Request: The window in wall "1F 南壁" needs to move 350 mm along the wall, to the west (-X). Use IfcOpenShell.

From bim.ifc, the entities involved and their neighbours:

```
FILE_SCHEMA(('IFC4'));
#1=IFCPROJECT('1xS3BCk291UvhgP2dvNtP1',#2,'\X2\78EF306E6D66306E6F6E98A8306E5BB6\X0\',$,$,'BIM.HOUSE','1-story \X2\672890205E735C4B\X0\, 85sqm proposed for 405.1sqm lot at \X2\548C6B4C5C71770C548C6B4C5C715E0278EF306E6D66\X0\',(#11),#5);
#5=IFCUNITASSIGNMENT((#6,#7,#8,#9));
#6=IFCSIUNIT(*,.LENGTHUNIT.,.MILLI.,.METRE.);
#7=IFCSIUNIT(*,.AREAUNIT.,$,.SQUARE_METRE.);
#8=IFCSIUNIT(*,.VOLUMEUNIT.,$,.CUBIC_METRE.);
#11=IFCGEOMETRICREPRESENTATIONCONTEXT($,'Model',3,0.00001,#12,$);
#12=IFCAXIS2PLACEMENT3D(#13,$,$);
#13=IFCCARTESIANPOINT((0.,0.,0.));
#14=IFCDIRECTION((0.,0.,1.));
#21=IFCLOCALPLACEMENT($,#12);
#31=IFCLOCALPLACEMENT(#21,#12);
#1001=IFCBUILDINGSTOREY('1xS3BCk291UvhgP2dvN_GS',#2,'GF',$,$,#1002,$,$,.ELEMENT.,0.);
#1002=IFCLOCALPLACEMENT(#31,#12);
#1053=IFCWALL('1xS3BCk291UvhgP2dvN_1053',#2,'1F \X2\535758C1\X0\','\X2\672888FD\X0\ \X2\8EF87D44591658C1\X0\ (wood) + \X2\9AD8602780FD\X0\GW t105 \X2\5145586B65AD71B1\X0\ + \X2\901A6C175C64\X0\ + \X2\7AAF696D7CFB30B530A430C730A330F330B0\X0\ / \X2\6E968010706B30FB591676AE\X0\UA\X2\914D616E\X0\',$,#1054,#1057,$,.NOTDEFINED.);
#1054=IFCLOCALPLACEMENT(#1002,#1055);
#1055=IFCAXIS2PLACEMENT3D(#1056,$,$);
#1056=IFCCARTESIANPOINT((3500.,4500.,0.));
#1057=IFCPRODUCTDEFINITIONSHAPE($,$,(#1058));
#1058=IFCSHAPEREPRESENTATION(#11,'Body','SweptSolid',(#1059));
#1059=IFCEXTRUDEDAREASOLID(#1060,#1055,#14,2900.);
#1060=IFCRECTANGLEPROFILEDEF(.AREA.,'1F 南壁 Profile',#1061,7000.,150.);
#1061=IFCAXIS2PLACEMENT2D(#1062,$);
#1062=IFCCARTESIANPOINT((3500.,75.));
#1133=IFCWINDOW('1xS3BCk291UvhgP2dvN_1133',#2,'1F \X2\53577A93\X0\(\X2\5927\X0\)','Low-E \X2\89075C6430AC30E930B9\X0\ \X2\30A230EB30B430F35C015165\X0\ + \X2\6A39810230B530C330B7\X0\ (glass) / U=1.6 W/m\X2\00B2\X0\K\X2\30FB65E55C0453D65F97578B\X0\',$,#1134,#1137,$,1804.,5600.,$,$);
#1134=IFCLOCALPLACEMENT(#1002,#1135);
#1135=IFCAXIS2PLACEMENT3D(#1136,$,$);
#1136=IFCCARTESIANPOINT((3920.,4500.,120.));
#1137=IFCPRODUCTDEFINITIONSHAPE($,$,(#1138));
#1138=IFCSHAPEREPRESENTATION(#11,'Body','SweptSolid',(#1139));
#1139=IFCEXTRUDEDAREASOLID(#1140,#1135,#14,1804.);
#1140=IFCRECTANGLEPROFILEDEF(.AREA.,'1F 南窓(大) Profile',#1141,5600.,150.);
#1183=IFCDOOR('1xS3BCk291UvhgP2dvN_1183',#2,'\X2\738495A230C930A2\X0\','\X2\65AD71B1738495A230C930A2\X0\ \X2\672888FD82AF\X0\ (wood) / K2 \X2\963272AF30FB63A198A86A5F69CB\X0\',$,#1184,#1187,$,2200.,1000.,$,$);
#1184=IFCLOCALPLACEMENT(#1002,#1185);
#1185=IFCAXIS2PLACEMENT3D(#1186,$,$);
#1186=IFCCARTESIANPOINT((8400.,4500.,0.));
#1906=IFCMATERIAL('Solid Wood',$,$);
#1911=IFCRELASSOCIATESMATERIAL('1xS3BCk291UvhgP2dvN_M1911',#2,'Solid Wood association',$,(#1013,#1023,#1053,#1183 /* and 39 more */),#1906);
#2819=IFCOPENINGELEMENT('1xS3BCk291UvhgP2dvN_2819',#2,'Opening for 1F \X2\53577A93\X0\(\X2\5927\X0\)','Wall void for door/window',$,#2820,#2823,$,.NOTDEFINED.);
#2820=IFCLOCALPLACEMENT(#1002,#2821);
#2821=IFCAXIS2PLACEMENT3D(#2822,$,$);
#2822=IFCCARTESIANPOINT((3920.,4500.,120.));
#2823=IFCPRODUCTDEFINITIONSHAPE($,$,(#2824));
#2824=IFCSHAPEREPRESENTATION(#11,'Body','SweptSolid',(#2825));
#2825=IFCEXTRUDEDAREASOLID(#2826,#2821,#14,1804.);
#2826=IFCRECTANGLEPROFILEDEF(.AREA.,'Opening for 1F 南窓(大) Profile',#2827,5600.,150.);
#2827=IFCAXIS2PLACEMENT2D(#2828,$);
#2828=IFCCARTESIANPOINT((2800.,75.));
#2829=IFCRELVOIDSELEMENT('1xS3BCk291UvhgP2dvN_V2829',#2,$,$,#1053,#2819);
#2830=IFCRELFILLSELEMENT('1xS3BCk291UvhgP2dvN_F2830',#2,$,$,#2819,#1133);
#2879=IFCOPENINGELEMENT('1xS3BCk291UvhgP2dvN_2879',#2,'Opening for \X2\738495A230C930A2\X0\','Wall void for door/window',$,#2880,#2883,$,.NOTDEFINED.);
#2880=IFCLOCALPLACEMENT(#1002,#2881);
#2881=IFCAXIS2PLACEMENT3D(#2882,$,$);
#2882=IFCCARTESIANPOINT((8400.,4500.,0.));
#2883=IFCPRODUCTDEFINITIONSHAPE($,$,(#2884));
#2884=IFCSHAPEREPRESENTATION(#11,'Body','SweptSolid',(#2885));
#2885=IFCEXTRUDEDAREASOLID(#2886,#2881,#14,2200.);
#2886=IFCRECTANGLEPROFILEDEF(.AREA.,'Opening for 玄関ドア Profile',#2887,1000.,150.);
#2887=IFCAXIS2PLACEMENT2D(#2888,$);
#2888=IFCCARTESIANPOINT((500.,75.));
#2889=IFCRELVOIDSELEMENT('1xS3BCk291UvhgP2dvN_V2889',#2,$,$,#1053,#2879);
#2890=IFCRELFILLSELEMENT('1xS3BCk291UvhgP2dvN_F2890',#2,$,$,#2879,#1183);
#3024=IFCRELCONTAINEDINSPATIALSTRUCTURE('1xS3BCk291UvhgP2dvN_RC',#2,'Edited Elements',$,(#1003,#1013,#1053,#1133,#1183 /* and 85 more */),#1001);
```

```python
import ifcopenshell
import ifcopenshell.api.geometry
import ifcopenshell.util.placement
import ifcopenshell.util.unit

model = ifcopenshell.open("bim.ifc")
unit_scale = ifcopenshell.util.unit.calculate_unit_scale(model)

window = model.by_guid("1xS3BCk291UvhgP2dvN_1133")
opening = window.FillsVoids[0].RelatingOpeningElement
wall = opening.VoidsElements[0].RelatingBuildingElement

wall_matrix = ifcopenshell.util.placement.get_local_placement(wall.ObjectPlacement)
shift = wall_matrix[:3, 0] * -0.35 / unit_scale
before = ifcopenshell.util.placement.get_local_placement(window.ObjectPlacement)[:3, 3].copy()

# The window is not placed relative to its opening, so move both.
for product in (opening, window):
    matrix = ifcopenshell.util.placement.get_local_placement(product.ObjectPlacement)
    matrix[:3, 3] += shift
    ifcopenshell.api.geometry.edit_object_placement(model, product=product, matrix=matrix, is_si=False)

after = ifcopenshell.util.placement.get_local_placement(window.ObjectPlacement)[:3, 3]
print("window moved by", (after - before).round(3) + 0.0)

model.write("bim_edited.ifc")
```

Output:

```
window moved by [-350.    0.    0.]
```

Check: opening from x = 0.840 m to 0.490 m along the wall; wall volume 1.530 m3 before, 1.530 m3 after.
